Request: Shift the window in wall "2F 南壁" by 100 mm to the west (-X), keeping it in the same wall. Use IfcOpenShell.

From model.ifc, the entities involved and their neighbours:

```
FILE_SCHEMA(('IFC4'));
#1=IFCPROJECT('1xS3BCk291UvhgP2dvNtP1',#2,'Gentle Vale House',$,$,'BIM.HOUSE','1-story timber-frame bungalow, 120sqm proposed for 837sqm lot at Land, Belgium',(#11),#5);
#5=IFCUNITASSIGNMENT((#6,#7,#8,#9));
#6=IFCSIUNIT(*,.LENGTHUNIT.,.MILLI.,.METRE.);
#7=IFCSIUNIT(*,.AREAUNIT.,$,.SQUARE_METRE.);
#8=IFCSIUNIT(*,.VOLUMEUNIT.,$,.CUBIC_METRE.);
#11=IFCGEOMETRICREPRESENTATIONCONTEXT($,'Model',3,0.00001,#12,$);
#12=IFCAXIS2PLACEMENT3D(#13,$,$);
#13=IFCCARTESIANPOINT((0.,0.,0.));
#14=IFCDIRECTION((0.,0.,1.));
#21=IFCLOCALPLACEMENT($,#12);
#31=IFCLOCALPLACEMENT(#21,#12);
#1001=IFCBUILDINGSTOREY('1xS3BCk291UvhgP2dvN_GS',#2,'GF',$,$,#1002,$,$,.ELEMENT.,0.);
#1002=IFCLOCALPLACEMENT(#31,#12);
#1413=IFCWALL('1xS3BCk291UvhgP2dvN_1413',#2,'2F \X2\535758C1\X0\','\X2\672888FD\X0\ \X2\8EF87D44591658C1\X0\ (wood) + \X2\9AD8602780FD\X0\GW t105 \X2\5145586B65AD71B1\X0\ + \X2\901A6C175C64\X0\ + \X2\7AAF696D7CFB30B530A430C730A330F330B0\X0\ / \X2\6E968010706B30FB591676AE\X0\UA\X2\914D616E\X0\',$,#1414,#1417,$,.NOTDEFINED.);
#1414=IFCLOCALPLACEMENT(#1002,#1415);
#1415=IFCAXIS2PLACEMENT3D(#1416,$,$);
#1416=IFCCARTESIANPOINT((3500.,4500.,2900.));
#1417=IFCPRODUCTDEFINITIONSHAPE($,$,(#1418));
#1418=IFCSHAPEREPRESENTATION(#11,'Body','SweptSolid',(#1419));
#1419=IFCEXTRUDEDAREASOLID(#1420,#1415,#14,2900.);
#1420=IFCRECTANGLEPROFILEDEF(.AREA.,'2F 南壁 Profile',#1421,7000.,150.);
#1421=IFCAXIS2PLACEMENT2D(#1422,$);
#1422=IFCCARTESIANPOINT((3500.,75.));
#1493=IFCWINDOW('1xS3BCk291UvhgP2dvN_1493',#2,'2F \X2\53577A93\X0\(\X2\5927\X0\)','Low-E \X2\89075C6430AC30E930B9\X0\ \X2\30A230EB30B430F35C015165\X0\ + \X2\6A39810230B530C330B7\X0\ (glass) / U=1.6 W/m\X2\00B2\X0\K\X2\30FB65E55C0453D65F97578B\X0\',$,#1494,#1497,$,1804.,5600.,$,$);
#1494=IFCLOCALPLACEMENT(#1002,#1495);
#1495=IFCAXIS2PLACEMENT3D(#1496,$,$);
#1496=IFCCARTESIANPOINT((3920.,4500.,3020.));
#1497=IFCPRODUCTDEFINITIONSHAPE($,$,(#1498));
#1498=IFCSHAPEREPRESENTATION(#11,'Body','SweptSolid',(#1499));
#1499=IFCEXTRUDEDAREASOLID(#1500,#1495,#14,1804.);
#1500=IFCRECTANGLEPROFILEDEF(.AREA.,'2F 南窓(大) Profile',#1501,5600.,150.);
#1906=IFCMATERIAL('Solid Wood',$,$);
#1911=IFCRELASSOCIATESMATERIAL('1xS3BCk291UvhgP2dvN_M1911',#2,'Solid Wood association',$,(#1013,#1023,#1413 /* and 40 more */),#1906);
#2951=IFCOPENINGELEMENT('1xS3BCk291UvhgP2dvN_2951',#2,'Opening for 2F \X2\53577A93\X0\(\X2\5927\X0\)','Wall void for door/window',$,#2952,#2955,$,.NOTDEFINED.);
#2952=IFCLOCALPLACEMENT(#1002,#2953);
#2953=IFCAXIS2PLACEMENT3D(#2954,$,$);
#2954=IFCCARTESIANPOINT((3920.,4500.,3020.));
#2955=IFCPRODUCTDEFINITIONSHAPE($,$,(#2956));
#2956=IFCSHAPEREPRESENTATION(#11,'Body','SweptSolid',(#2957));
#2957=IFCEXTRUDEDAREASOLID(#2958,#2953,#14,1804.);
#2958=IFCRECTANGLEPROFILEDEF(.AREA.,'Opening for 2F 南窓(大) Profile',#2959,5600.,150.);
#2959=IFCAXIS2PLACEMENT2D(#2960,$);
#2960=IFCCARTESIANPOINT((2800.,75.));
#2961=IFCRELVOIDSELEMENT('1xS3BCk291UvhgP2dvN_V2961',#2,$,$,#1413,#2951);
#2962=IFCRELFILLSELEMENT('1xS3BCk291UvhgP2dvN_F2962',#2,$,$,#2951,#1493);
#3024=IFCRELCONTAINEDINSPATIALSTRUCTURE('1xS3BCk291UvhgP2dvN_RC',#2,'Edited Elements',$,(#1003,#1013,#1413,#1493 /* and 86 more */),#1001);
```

```python
import ifcopenshell
import ifcopenshell.api.geometry
import ifcopenshell.util.placement
import ifcopenshell.util.unit

model = ifcopenshell.open("model.ifc")
unit_scale = ifcopenshell.util.unit.calculate_unit_scale(model)

window = model.by_guid("1xS3BCk291UvhgP2dvN_1493")
opening = window.FillsVoids[0].RelatingOpeningElement
wall = opening.VoidsElements[0].RelatingBuildingElement

wall_matrix = ifcopenshell.util.placement.get_local_placement(wall.ObjectPlacement)
shift = wall_matrix[:3, 0] * -0.1 / unit_scale
before = ifcopenshell.util.placement.get_local_placement(window.ObjectPlacement)[:3, 3].copy()

# The window is not placed relative to its opening, so move both.
for product in (opening, window):
    matrix = ifcopenshell.util.placement.get_local_placement(product.ObjectPlacement)
    matrix[:3, 3] += shift
    ifcopenshell.api.geometry.edit_object_placement(model, product=product, matrix=matrix, is_si=False)

after = ifcopenshell.util.placement.get_local_placement(window.ObjectPlacement)[:3, 3]
print("window moved by", (after - before).round(3) + 0.0)

model.write("model_rev.ifc")
```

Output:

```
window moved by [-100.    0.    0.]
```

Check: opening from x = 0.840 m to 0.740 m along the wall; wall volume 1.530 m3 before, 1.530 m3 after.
